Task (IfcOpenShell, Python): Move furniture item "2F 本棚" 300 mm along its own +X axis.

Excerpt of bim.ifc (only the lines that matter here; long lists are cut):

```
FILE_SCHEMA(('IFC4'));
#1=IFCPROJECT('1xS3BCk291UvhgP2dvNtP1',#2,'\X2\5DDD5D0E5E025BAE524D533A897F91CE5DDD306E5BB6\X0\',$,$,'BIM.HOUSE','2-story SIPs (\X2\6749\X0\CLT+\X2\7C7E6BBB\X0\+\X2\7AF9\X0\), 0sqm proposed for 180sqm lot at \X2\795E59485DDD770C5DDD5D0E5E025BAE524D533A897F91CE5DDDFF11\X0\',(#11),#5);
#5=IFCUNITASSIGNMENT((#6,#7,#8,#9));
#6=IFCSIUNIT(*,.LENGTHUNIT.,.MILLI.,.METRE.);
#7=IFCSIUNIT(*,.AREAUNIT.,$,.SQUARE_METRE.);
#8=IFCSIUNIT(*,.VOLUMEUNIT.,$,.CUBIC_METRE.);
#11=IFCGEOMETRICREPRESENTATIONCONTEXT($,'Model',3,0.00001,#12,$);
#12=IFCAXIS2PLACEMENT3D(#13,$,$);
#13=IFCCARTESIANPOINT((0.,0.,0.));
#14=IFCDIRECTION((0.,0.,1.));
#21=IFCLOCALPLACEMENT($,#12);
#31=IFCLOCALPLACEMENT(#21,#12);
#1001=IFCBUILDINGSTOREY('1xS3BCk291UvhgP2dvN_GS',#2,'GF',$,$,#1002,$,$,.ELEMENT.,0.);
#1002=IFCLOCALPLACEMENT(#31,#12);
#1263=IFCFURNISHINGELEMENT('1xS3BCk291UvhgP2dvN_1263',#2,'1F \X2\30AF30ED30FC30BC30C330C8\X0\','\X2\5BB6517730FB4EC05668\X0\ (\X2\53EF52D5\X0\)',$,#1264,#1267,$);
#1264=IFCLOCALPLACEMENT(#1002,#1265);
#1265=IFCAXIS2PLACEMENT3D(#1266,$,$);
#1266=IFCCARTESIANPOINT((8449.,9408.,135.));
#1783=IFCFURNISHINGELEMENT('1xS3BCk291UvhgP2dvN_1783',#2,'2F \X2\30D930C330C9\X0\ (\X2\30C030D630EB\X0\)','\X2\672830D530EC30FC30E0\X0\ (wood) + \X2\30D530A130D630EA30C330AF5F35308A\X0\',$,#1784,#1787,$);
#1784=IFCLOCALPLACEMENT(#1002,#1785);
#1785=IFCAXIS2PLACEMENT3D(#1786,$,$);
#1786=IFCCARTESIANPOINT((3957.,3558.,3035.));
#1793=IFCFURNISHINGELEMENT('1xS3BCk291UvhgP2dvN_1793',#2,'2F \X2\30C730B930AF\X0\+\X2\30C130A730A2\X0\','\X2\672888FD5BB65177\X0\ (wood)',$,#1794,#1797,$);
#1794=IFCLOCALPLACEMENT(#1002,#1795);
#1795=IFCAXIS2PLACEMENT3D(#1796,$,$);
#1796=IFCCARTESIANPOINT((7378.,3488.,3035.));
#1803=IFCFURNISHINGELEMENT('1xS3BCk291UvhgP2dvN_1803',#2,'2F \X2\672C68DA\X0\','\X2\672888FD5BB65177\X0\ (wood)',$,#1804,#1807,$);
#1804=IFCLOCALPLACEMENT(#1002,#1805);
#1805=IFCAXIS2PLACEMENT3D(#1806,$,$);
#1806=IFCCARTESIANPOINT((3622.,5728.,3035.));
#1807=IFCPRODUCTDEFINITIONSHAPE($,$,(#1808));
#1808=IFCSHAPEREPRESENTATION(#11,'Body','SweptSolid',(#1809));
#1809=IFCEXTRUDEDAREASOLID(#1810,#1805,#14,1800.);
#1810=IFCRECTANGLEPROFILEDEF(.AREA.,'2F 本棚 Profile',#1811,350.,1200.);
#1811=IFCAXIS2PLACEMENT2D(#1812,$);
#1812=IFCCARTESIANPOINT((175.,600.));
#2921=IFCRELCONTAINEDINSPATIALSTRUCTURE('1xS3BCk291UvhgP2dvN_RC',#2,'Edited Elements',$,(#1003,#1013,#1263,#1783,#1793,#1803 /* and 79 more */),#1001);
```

```python
import ifcopenshell
import ifcopenshell.api.geometry
import ifcopenshell.util.placement
import ifcopenshell.util.unit

model = ifcopenshell.open("bim.ifc")
unit_scale = ifcopenshell.util.unit.calculate_unit_scale(model)

item = model.by_guid("1xS3BCk291UvhgP2dvN_1803")
matrix = ifcopenshell.util.placement.get_local_placement(item.ObjectPlacement)
matrix[:3, 3] += matrix[:3, 0] * 0.3 / unit_scale
ifcopenshell.api.geometry.edit_object_placement(model, product=item, matrix=matrix, is_si=False)

print(ifcopenshell.util.placement.get_local_placement(item.ObjectPlacement).round(3) + 0.0)

model.write("bim_updated.ifc")
```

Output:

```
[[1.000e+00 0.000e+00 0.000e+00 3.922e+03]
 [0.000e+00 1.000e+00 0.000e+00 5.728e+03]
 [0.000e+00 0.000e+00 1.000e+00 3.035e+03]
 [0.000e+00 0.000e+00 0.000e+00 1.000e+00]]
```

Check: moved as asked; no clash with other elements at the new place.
